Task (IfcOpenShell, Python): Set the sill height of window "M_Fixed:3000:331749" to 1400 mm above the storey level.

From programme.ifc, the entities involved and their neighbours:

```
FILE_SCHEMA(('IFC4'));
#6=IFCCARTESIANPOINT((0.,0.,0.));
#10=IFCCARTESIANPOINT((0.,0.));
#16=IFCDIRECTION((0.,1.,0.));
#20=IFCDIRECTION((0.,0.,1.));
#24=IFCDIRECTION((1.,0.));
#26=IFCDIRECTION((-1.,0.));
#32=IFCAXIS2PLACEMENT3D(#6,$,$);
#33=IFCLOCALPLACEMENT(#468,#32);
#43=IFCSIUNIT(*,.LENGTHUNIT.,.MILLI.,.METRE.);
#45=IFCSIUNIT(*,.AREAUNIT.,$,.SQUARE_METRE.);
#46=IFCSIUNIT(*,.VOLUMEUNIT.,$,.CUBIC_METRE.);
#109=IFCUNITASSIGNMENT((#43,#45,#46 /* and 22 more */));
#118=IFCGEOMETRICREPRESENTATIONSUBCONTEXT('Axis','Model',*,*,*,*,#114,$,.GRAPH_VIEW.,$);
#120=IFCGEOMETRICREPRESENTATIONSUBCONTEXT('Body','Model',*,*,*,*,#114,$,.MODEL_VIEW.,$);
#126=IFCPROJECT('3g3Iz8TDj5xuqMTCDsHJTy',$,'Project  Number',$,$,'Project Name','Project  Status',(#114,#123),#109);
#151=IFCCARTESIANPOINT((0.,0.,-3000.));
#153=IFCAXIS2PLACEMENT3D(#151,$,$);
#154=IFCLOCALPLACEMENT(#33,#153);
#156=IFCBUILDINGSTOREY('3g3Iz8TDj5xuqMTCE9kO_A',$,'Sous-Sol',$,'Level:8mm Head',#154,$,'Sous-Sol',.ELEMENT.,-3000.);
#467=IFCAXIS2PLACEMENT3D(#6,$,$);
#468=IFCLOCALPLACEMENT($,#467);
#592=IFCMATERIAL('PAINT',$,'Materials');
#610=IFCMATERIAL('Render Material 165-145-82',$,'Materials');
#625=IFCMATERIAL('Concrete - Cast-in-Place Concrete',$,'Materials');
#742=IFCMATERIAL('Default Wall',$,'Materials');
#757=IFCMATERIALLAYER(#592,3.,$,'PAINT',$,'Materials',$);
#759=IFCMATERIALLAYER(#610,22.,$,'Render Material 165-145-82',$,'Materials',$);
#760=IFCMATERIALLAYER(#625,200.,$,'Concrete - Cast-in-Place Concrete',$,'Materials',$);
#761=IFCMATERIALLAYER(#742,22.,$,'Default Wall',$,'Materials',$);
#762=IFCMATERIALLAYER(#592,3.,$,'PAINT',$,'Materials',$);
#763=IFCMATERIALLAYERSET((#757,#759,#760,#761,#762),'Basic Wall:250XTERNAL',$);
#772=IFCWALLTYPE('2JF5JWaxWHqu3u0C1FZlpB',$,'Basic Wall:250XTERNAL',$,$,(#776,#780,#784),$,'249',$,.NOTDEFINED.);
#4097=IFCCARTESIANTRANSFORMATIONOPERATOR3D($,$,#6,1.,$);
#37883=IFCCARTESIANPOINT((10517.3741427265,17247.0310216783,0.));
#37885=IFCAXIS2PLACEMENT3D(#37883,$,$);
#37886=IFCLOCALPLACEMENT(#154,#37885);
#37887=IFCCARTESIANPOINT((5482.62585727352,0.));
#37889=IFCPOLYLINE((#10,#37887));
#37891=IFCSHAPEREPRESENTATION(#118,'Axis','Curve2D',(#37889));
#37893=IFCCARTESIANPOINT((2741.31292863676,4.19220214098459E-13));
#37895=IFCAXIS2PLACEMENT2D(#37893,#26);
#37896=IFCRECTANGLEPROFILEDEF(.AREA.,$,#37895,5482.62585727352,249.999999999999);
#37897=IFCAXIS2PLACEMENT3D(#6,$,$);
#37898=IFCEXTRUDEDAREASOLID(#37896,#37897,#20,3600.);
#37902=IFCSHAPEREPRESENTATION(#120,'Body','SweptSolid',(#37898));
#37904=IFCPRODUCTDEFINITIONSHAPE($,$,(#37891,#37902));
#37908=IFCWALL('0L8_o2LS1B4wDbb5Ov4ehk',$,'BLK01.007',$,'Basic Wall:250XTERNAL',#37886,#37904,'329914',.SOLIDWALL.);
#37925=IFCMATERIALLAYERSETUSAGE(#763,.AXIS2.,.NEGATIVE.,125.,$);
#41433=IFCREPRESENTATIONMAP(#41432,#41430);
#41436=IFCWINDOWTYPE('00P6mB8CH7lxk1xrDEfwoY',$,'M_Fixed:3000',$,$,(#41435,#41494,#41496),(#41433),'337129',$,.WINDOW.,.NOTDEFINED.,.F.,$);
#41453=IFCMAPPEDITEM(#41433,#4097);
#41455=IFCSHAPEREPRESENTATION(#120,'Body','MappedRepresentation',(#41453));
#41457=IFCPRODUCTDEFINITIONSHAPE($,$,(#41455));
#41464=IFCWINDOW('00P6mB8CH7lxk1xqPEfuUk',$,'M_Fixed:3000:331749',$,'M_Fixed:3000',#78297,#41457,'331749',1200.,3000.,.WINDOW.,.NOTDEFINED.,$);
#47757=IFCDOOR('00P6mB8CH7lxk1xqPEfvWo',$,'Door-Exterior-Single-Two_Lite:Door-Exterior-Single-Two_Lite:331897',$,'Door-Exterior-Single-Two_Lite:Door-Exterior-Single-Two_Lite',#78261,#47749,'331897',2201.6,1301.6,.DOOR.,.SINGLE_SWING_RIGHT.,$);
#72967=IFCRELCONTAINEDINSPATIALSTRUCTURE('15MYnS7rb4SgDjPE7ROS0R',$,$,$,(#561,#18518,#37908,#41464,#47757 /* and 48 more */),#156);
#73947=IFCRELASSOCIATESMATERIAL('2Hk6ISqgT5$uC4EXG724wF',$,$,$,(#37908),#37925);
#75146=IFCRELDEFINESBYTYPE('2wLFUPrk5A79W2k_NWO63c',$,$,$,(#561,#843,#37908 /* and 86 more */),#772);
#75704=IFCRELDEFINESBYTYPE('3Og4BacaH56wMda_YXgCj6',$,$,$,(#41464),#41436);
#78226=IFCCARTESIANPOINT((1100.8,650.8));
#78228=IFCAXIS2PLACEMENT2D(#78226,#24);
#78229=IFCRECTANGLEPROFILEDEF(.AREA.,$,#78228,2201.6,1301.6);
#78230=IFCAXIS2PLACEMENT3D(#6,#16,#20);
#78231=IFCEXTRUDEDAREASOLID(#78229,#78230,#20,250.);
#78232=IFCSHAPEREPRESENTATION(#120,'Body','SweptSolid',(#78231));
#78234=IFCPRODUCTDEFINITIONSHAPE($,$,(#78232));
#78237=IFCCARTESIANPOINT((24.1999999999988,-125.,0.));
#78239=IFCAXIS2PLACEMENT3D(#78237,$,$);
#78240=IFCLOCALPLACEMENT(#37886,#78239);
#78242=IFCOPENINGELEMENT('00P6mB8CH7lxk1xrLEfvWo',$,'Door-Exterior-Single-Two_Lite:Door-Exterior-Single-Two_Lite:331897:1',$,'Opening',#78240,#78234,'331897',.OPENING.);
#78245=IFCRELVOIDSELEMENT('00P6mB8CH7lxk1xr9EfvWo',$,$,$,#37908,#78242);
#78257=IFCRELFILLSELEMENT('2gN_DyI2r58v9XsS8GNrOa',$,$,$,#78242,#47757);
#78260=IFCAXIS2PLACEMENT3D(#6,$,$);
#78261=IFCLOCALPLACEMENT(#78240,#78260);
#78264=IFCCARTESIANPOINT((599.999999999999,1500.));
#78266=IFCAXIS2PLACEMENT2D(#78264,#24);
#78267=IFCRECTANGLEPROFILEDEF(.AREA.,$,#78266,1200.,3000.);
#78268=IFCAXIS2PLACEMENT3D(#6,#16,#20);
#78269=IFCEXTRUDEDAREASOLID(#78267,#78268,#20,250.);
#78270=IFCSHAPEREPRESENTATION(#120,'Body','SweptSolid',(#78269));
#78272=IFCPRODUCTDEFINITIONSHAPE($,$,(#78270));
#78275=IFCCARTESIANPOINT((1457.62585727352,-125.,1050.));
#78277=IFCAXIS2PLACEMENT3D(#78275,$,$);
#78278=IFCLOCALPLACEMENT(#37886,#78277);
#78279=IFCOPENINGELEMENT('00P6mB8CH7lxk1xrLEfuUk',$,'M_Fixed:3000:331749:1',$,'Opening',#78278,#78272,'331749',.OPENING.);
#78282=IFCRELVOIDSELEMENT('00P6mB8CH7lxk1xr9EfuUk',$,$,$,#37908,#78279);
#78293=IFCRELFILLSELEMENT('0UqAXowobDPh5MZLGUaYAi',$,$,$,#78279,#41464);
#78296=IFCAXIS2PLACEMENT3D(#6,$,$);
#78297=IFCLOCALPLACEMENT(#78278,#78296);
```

```python
import numpy as np
import ifcopenshell
import ifcopenshell.api.geometry
import ifcopenshell.geom
import ifcopenshell.util.element
import ifcopenshell.util.placement
import ifcopenshell.util.shape
import ifcopenshell.util.unit

model = ifcopenshell.open("programme.ifc")
unit_scale = ifcopenshell.util.unit.calculate_unit_scale(model)

window = model.by_guid("00P6mB8CH7lxk1xqPEfuUk")
opening = window.FillsVoids[0].RelatingOpeningElement
storey = ifcopenshell.util.element.get_container(window, ifc_class="IfcBuildingStorey")
level = ifcopenshell.util.placement.get_local_placement(storey.ObjectPlacement)[2, 3]

# The opening's origin need not be at the sill, so measure its lowest point.
shape = ifcopenshell.geom.create_shape(ifcopenshell.geom.settings(), opening)
bottom = ifcopenshell.util.shape.get_shape_bottom_elevation(shape, shape.geometry) / unit_scale
dz = level + 1.4 / unit_scale - bottom

shift = np.array([0.0, 0.0, dz])
# The window is placed relative to its opening, so it follows when the opening moves.
matrix = ifcopenshell.util.placement.get_local_placement(opening.ObjectPlacement)
matrix[:3, 3] += shift
ifcopenshell.api.geometry.edit_object_placement(
    model, product=opening, matrix=matrix, is_si=False, should_transform_children=True
)

print(f"moved by {dz * unit_scale:+.3f} m")

model.write("programme_v2.ifc")
```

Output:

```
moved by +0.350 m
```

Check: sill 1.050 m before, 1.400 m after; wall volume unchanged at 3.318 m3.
